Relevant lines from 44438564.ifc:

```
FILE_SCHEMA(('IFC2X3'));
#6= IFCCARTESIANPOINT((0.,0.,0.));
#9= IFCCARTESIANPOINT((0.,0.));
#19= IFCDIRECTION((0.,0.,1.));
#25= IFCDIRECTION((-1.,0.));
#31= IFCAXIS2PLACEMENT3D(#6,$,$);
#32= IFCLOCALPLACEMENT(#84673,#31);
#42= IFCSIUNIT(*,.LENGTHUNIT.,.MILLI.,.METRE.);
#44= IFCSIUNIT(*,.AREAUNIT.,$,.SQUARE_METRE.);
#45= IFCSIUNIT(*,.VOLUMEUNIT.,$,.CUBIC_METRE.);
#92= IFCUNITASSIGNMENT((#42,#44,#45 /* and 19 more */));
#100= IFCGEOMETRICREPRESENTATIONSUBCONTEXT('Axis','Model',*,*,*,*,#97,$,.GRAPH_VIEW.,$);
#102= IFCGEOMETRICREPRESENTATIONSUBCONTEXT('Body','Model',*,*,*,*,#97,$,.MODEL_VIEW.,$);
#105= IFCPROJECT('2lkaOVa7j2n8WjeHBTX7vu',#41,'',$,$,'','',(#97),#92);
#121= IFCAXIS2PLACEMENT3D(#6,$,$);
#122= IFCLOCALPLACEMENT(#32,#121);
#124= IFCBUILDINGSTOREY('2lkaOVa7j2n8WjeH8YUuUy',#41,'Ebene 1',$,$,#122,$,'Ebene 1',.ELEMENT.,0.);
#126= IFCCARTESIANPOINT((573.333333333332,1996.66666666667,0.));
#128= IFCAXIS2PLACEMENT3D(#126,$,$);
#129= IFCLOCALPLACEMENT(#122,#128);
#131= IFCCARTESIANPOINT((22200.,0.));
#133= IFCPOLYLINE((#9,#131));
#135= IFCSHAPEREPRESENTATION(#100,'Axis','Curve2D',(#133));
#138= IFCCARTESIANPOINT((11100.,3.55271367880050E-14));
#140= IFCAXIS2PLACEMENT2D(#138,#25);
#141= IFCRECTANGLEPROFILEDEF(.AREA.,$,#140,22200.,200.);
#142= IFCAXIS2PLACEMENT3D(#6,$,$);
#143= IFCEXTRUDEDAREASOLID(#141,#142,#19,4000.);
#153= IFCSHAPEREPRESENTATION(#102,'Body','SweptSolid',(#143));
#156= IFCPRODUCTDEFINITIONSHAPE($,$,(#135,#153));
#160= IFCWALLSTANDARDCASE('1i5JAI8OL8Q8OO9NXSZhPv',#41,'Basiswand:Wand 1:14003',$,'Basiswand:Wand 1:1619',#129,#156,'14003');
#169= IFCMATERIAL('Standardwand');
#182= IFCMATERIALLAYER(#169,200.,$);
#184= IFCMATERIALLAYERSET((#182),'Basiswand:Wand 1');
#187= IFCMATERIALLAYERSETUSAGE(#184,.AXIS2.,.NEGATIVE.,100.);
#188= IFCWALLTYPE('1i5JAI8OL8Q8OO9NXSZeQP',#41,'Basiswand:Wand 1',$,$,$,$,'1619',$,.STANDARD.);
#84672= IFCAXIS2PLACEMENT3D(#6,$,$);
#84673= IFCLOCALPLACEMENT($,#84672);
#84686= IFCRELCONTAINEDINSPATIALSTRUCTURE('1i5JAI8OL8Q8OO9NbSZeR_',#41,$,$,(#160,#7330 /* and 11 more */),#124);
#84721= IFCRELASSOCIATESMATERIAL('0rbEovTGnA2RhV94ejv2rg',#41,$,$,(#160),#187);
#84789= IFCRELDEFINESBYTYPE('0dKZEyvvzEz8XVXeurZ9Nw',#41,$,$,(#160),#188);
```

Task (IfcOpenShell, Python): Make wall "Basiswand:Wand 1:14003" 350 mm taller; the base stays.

```python
import ifcopenshell
import ifcopenshell.geom
import ifcopenshell.util.representation
import ifcopenshell.util.shape

model = ifcopenshell.open("44438564.ifc")
settings = ifcopenshell.geom.settings()


def volume(element):
    """Net volume in cubic metres, openings subtracted."""
    shape = ifcopenshell.geom.create_shape(settings, element)
    return ifcopenshell.util.shape.get_volume(shape.geometry)


wall = model.by_guid("1i5JAI8OL8Q8OO9NXSZhPv")
before = volume(wall)

body = ifcopenshell.util.representation.get_representation(wall, "Model", "Body")
solid = body.Items[0]
old_height = solid.Depth
solid.Depth += 350.0
after = volume(wall)

print(f"height {old_height:g} -> {solid.Depth:g}, volume {before:.3f} -> {after:.3f} m3")

model.write("44438564_edited.ifc")
```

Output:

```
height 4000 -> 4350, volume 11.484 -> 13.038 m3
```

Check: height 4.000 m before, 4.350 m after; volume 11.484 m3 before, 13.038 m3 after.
